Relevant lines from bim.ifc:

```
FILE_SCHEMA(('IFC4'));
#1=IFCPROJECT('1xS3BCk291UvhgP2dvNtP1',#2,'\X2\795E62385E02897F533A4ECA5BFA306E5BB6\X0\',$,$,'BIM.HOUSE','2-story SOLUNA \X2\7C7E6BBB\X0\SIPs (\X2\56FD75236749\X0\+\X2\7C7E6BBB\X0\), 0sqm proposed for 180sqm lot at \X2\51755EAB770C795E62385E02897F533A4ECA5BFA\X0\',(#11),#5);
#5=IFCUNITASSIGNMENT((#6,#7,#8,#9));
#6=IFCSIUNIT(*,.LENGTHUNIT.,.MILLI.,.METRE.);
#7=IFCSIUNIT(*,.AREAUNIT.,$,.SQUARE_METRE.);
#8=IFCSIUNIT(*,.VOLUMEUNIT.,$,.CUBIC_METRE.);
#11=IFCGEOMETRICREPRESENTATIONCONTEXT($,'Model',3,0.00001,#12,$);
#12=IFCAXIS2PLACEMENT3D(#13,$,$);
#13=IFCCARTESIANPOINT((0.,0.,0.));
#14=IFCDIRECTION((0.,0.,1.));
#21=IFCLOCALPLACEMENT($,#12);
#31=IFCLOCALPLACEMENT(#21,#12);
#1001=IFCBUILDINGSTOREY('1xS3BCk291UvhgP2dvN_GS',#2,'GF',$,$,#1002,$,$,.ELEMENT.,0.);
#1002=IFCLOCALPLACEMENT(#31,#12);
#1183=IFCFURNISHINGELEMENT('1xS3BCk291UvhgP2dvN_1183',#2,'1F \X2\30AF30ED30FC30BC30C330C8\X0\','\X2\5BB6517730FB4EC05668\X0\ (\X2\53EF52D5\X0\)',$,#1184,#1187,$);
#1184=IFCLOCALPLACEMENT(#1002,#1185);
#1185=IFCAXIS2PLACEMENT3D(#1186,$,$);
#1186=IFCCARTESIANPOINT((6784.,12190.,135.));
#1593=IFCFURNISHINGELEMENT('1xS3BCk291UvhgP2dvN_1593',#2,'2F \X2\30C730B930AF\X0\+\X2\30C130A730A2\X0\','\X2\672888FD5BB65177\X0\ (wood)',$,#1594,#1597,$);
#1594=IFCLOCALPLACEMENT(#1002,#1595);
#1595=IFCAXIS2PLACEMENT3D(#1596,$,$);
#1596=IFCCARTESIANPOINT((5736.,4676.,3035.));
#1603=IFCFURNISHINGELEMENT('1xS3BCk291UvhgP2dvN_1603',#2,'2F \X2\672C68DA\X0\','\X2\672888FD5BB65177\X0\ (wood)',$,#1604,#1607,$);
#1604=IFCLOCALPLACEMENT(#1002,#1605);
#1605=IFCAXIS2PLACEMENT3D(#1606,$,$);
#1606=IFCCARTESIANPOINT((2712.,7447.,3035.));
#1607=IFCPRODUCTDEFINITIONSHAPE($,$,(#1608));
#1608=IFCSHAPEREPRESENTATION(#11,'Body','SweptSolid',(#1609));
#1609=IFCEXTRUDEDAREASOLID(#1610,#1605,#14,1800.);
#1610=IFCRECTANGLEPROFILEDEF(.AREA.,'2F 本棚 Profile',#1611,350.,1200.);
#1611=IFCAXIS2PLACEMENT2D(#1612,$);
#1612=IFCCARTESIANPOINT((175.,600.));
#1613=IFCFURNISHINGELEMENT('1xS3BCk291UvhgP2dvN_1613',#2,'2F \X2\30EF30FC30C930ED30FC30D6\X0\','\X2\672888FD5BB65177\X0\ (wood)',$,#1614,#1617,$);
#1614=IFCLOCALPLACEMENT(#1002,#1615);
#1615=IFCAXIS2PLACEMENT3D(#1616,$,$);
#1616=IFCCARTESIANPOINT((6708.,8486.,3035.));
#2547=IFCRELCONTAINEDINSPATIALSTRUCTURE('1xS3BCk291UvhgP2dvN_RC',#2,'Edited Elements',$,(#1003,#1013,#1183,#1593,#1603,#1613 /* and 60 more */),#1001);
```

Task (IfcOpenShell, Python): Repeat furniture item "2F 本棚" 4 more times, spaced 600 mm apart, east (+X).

```python
import numpy as np
import ifcopenshell
import ifcopenshell.api.geometry
import ifcopenshell.api.root
import ifcopenshell.util.element
import ifcopenshell.util.placement
import ifcopenshell.util.unit

model = ifcopenshell.open("bim.ifc")
unit_scale = ifcopenshell.util.unit.calculate_unit_scale(model)


def reuse_history(source, copy):
    """copy_class also copies each property set's owner history, people and application; keep the originals."""
    for rel in copy.IsDefinedBy:
        if rel.is_a("IfcRelDefinesByProperties") and (history := rel.RelatingPropertyDefinition.OwnerHistory):
            rel.RelatingPropertyDefinition.OwnerHistory = source.OwnerHistory
            ifcopenshell.util.element.remove_deep2(model, history)


source = model.by_guid("1xS3BCk291UvhgP2dvN_1603")
base = ifcopenshell.util.placement.get_local_placement(source.ObjectPlacement)
step = np.array([1.0, 0.0, 0.0]) * 0.6 / unit_scale

for i in range(1, 5):
    copy = ifcopenshell.api.root.copy_class(model, product=source)
    copy.Representation = ifcopenshell.util.element.copy_deep(
        model, source.Representation, exclude=["IfcGeometricRepresentationContext", "IfcRepresentationMap"]
    )
    reuse_history(source, copy)
    matrix = base.copy()
    matrix[:3, 3] += i * step
    print("added at", matrix[:3, 3].round(3) + 0.0)
    ifcopenshell.api.geometry.edit_object_placement(model, product=copy, matrix=matrix, is_si=False)

model.write("bim_edited.ifc")
```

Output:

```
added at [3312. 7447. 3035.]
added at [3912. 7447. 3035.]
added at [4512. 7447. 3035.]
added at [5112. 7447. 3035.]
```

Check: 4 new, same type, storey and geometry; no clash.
